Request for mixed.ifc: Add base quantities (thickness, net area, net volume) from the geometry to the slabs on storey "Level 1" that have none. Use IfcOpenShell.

First a look at what the model holds.

```python
import ifcopenshell
import ifcopenshell.util.element
import ifcopenshell.util.unit

model = ifcopenshell.open("mixed.ifc")
print(model.schema)
for unit_type in ("LENGTHUNIT", "AREAUNIT", "VOLUMEUNIT"):
    print(unit_type, ifcopenshell.util.unit.calculate_unit_scale(model, unit_type))
storey = next(s for s in model.by_type("IfcBuildingStorey") if s.Name == "Level 1")
slabs = [e for e in ifcopenshell.util.element.get_decomposition(storey) if e.is_a("IfcSlab")]
for e in sorted(slabs, key=lambda e: e.id()):
    print(e.id(), e.is_a(), e.Name, list(ifcopenshell.util.element.get_psets(e, qtos_only=True)), sep=" | ")
```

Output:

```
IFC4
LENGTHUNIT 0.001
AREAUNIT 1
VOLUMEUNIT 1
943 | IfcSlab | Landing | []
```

```python
import ifcopenshell
import ifcopenshell.api.pset
import ifcopenshell.geom
import ifcopenshell.util.element
import ifcopenshell.util.shape
import ifcopenshell.util.unit

model = ifcopenshell.open("mixed.ifc")
unit_scale = ifcopenshell.util.unit.calculate_unit_scale(model)
area_scale = ifcopenshell.util.unit.calculate_unit_scale(model, "AREAUNIT")
volume_scale = ifcopenshell.util.unit.calculate_unit_scale(model, "VOLUMEUNIT")
settings = ifcopenshell.geom.settings()

storey = next(s for s in model.by_type("IfcBuildingStorey") if s.Name == "Level 1")
slabs = [e for e in ifcopenshell.util.element.get_decomposition(storey) if e.is_a("IfcSlab")]

for e in sorted(slabs, key=lambda e: e.id()):
    if ifcopenshell.util.element.get_psets(e, qtos_only=True, should_inherit=False):
        continue
    # Geometry comes back in metres, in the element's own axes.
    shape = ifcopenshell.geom.create_shape(settings, e)
    values = {
        "Width": ifcopenshell.util.shape.get_z(shape.geometry) / unit_scale,
        "NetArea": ifcopenshell.util.shape.get_footprint_area(shape.geometry) / area_scale,
        "NetVolume": ifcopenshell.util.shape.get_volume(shape.geometry) / volume_scale,
    }
    qto = ifcopenshell.api.pset.add_qto(model, product=e, name="Qto_SlabBaseQuantities")
    ifcopenshell.api.pset.edit_qto(model, qto=qto, properties=values)
    print(e.id(), {k: round(v, 3) for k, v in values.items()})

model.write("mixed-out.ifc")
```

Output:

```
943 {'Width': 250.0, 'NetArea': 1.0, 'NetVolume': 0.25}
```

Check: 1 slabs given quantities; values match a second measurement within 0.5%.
